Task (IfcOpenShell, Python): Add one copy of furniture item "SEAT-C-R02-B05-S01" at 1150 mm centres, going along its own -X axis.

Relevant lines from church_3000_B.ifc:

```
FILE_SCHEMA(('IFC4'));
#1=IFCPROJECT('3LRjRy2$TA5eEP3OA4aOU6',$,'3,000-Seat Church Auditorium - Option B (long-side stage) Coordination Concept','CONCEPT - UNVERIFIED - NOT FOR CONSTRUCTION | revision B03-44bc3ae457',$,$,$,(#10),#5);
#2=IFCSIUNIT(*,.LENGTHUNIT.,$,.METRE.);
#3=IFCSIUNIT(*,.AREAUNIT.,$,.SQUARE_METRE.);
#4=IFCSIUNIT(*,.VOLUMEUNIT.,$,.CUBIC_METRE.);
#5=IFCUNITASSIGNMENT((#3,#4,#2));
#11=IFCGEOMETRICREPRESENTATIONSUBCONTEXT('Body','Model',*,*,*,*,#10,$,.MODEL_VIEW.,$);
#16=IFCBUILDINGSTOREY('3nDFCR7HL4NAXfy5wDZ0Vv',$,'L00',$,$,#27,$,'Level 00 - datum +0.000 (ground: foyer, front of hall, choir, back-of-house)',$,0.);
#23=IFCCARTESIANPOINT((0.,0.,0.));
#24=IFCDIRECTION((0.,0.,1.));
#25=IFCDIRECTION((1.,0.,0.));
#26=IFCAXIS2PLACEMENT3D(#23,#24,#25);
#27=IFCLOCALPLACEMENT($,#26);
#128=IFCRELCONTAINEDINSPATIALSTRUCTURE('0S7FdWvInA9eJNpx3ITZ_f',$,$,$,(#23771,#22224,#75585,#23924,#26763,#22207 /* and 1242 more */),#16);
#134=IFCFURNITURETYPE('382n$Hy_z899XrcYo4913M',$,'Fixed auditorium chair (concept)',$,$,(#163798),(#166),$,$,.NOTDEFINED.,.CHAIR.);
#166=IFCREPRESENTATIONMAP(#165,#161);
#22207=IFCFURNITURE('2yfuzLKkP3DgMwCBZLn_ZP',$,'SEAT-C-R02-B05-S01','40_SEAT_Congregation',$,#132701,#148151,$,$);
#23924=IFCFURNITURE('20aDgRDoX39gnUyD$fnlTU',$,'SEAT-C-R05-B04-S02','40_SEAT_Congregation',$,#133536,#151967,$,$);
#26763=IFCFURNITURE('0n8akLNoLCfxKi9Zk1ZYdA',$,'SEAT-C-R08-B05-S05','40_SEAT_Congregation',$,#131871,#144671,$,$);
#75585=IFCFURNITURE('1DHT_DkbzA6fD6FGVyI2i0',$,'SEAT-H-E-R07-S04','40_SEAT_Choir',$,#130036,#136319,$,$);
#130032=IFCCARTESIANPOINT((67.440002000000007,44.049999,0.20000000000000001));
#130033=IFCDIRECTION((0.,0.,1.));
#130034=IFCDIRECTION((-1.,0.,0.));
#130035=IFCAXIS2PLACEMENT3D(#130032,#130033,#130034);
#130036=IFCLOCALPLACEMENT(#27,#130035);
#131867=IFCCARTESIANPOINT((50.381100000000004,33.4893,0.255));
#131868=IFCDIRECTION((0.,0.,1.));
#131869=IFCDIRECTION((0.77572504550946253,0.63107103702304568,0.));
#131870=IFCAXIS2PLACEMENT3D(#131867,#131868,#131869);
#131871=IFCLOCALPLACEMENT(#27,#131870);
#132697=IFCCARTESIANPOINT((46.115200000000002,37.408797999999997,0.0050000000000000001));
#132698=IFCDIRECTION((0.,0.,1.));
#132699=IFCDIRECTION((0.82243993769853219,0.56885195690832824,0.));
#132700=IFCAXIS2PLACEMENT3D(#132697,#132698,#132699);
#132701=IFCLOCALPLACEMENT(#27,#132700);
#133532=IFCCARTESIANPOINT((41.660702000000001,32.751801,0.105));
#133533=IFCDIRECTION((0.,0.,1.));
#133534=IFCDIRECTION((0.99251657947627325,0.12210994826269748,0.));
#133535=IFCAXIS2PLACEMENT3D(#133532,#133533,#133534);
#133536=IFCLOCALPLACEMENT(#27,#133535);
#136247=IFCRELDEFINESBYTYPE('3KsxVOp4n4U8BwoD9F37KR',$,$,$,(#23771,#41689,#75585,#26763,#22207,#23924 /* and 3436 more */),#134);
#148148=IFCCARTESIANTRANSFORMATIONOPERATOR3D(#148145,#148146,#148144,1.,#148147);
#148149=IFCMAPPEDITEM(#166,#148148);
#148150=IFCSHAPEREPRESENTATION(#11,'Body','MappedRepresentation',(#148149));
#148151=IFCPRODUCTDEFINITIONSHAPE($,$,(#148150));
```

```python
import ifcopenshell
import ifcopenshell.api.geometry
import ifcopenshell.api.root
import ifcopenshell.util.element
import ifcopenshell.util.placement

model = ifcopenshell.open("church_3000_B.ifc")

source = model.by_guid("2yfuzLKkP3DgMwCBZLn_ZP")
base = ifcopenshell.util.placement.get_local_placement(source.ObjectPlacement)
step = -base[:3, 0] * 1.15

for i in range(1, 2):
    copy = ifcopenshell.api.root.copy_class(model, product=source)
    copy.Representation = ifcopenshell.util.element.copy_deep(
        model, source.Representation, exclude=["IfcGeometricRepresentationContext", "IfcRepresentationMap"]
    )
    matrix = base.copy()
    matrix[:3, 3] += i * step
    print("added at", matrix[:3, 3].round(3) + 0.0)
    ifcopenshell.api.geometry.edit_object_placement(model, product=copy, matrix=matrix, is_si=False)

model.write("church_3000_B-out.ifc")
```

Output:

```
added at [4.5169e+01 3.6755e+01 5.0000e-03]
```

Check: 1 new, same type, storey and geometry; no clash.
